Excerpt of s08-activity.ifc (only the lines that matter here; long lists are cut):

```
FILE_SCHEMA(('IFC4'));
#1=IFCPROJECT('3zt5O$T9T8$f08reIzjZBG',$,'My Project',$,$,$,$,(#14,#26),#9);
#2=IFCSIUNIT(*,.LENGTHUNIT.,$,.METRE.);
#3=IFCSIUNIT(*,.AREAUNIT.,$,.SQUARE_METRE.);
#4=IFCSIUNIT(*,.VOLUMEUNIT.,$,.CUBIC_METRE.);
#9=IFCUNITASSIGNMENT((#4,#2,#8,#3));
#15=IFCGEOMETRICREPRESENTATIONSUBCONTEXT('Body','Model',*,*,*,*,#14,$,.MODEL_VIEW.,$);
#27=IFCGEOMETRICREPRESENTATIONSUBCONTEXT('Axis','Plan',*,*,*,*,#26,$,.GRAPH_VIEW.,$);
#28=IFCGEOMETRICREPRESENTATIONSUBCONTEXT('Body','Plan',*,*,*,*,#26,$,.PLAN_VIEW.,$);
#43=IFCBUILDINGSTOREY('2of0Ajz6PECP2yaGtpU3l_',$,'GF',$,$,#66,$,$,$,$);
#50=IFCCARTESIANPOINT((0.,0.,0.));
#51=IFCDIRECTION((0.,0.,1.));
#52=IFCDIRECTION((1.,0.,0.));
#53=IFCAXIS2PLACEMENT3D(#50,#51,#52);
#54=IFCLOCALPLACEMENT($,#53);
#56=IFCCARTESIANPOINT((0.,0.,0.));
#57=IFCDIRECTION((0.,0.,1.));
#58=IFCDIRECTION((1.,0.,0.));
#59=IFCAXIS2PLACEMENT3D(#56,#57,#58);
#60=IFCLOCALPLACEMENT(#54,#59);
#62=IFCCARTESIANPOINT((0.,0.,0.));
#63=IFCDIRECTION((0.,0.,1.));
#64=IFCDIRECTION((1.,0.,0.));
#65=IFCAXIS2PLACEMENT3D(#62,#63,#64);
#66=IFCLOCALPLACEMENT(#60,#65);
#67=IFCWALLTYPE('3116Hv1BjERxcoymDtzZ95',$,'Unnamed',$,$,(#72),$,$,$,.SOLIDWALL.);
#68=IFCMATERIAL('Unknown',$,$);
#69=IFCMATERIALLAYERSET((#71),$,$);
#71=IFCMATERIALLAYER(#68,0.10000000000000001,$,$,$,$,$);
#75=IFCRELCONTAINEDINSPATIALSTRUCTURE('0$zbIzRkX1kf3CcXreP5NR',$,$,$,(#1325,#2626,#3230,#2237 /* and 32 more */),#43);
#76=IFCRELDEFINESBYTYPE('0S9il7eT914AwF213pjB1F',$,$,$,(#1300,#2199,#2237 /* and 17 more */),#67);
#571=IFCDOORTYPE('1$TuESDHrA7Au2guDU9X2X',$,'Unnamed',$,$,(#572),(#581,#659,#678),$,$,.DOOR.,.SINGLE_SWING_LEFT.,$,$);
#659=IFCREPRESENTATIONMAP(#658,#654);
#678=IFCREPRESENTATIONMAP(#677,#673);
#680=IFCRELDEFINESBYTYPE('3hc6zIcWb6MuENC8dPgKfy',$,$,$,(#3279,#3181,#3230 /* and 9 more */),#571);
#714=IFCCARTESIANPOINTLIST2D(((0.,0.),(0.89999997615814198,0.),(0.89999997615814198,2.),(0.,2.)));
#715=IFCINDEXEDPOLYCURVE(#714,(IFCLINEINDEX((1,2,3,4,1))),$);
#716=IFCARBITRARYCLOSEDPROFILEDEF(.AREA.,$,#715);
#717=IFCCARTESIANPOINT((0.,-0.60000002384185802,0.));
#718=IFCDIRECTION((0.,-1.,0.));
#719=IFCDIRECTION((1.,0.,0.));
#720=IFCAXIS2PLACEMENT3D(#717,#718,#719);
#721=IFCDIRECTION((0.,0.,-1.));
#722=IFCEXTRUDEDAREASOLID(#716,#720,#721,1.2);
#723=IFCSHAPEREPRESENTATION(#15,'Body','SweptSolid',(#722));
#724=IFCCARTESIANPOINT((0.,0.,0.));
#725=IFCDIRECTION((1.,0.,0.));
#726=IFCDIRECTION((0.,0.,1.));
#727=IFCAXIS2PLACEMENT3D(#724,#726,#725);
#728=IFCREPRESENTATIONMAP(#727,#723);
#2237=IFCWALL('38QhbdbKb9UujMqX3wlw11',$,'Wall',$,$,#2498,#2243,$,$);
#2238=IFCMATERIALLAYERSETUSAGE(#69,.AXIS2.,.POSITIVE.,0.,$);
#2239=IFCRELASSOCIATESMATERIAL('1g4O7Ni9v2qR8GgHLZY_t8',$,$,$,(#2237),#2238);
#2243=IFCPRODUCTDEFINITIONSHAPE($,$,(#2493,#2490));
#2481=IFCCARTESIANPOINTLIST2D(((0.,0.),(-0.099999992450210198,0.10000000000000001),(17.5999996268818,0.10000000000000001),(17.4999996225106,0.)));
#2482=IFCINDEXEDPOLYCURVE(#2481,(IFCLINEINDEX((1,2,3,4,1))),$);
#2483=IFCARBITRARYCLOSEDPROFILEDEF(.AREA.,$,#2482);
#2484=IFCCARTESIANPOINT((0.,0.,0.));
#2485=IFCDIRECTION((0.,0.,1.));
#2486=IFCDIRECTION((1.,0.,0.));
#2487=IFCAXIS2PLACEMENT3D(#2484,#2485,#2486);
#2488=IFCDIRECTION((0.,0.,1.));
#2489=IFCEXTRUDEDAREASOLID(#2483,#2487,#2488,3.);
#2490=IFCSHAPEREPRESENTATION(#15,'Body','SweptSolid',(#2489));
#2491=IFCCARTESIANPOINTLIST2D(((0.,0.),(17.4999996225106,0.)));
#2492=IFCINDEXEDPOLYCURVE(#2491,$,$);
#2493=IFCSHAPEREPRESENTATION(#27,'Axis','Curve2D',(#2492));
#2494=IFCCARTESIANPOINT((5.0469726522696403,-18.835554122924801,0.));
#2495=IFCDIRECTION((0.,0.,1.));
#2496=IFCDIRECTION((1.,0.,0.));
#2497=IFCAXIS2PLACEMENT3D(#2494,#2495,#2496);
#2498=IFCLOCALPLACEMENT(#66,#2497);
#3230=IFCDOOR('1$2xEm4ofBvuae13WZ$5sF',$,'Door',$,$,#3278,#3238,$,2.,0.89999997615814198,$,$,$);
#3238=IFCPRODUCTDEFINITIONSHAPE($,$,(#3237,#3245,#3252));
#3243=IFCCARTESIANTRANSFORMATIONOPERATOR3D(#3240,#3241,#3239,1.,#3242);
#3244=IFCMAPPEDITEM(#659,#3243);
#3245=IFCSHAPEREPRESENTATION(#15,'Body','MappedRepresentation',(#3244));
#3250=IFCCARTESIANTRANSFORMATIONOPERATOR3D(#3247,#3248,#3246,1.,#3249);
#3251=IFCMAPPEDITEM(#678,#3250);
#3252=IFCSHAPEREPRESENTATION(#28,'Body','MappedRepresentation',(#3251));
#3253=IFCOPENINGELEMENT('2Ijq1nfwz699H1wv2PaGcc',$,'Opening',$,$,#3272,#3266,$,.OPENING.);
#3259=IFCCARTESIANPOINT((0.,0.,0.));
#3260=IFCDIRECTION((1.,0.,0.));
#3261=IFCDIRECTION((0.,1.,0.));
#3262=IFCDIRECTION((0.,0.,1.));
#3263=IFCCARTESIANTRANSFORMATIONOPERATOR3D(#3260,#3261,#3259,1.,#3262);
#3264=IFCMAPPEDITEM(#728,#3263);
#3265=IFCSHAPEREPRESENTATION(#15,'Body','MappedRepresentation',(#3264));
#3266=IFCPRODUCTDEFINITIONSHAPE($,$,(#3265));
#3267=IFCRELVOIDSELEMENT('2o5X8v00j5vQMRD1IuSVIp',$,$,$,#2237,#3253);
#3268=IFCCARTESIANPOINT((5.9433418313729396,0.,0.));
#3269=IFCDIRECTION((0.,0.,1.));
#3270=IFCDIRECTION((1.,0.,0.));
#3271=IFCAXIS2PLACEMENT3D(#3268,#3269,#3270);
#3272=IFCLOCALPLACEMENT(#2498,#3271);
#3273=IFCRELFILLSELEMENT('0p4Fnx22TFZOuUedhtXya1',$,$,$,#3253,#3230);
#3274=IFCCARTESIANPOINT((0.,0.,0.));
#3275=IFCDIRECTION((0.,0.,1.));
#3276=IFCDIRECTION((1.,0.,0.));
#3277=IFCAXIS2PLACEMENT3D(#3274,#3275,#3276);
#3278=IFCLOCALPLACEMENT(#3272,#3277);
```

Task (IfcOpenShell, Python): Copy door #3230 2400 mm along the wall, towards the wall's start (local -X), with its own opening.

```python
import ifcopenshell
import ifcopenshell.api.feature
import ifcopenshell.api.geometry
import ifcopenshell.api.root
import ifcopenshell.geom
import ifcopenshell.util.element
import ifcopenshell.util.placement
import ifcopenshell.util.shape

model = ifcopenshell.open("s08-activity.ifc")
settings = ifcopenshell.geom.settings()


def volume(element):
    """Net volume in cubic metres, openings subtracted."""
    shape = ifcopenshell.geom.create_shape(settings, element)
    return ifcopenshell.util.shape.get_volume(shape.geometry)


door = model.by_guid("1$2xEm4ofBvuae13WZ$5sF")
opening = door.FillsVoids[0].RelatingOpeningElement
wall = opening.VoidsElements[0].RelatingBuildingElement
before = volume(wall)
shift = ifcopenshell.util.placement.get_local_placement(wall.ObjectPlacement)[:3, 0] * -2.4

# copy_class copies the void relationship, type, container and properties, but no geometry.
new_opening = ifcopenshell.api.root.copy_class(model, product=opening)
new_opening.Representation = ifcopenshell.util.element.copy_deep(
    model, opening.Representation, exclude=["IfcGeometricRepresentationContext", "IfcRepresentationMap"]
)
new_door = ifcopenshell.api.root.copy_class(model, product=door)
new_door.Representation = ifcopenshell.util.element.copy_deep(
    model, door.Representation, exclude=["IfcGeometricRepresentationContext", "IfcRepresentationMap"]
)
ifcopenshell.api.feature.add_filling(model, opening=new_opening, element=new_door)

for old, new in ((opening, new_opening), (door, new_door)):
    matrix = ifcopenshell.util.placement.get_local_placement(old.ObjectPlacement)
    matrix[:3, 3] += shift
    ifcopenshell.api.geometry.edit_object_placement(model, product=new, matrix=matrix, is_si=False)

after = volume(wall)

print(f"wall volume {before:.3f} -> {after:.3f} m3")

model.write("s08-activity_v2.ifc")
```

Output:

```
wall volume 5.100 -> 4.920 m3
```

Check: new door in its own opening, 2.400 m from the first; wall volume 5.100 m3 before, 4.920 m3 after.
